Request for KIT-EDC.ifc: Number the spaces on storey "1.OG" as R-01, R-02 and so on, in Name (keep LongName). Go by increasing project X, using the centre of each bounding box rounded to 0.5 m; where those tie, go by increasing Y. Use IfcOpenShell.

First a look at what the model holds.

```python
import ifcopenshell
import ifcopenshell.util.element
import ifcopenshell.util.placement

model = ifcopenshell.open("KIT-EDC.ifc")
print(model.schema)
storey = next(s for s in model.by_type("IfcBuildingStorey") if s.Name == "1.OG")
spaces = [e for e in ifcopenshell.util.element.get_decomposition(storey) if e.is_a("IfcSpace")]
for e in sorted(spaces, key=lambda e: e.id()):
    origin = ifcopenshell.util.placement.get_local_placement(e.ObjectPlacement)[:3, 3]
    print(e.id(), e.Name, e.LongName, origin.round(2) + 0.0, sep=" | ")
```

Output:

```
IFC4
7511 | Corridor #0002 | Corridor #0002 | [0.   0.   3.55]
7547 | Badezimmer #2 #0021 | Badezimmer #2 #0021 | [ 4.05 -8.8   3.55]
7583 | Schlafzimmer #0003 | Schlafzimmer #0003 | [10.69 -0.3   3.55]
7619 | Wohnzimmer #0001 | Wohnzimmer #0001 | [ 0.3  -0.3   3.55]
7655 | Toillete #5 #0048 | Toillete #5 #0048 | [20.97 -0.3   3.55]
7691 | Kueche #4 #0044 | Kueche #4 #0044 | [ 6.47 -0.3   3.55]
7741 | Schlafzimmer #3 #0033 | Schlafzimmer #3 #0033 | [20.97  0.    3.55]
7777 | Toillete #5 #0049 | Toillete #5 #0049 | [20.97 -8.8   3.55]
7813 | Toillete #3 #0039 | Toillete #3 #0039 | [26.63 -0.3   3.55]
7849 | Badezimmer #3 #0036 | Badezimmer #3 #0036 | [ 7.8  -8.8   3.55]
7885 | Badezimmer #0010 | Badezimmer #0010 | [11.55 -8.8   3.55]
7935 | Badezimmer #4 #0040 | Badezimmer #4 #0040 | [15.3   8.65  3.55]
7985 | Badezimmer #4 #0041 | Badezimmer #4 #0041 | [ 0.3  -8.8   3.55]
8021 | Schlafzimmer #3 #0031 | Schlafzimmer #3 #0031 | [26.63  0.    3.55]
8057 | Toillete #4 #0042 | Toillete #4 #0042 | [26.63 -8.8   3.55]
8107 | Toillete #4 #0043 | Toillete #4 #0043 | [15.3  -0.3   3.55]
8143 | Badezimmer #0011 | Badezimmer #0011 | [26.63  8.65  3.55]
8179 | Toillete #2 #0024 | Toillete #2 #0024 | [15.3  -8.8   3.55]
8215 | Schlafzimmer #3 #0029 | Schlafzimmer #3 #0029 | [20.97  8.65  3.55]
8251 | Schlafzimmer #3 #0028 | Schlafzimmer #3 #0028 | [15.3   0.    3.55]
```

```python
import ifcopenshell
import ifcopenshell.geom
import ifcopenshell.util.element
import ifcopenshell.util.shape

model = ifcopenshell.open("KIT-EDC.ifc")
settings = ifcopenshell.geom.settings()
settings.set("use-world-coords", True)


def centre(element):
    shape = ifcopenshell.geom.create_shape(settings, element)
    return ifcopenshell.util.shape.get_bbox_centroid(shape.geometry)


storey = next(s for s in model.by_type("IfcBuildingStorey") if s.Name == "1.OG")
spaces = [e for e in ifcopenshell.util.element.get_decomposition(storey) if e.is_a("IfcSpace")]

# Insertion points can sit at a corner or the storey origin, so sort by the geometry (in metres).
centres = {e: centre(e) for e in spaces}
spaces.sort(key=lambda e: (round(centres[e][0] / 0.5), centres[e][1]))

for i, e in enumerate(spaces, start=1):
    number = f"R-{i:02d}"
    e.Name = number
    print(e.id(), number)

model.write("KIT-EDC_v2.ifc")
```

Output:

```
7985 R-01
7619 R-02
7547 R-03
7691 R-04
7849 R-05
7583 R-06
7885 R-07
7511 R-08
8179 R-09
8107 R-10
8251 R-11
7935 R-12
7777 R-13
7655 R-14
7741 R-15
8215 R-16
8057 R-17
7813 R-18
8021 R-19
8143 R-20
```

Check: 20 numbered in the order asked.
